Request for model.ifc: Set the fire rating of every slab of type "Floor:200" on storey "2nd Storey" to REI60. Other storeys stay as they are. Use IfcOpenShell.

First a look at what the model holds.

```python
import ifcopenshell
import ifcopenshell.util.element

model = ifcopenshell.open("model.ifc")
print(model.schema)
storey = next(s for s in model.by_type("IfcBuildingStorey") if s.Name == "2nd Storey")
slabs = [e for e in ifcopenshell.util.element.get_decomposition(storey) if e.is_a("IfcSlab")]
seen = {}
for e in slabs:
    element_type = ifcopenshell.util.element.get_type(e)
    key = (element_type.Name if element_type != e and element_type else None, ifcopenshell.util.element.get_pset(e, "Pset_SlabCommon", "FireRating"))
    seen[key] = seen.get(key, 0) + 1
for (name, value), count in sorted(seen.items(), key=str):
    print(count, "x", name, "|", value)
```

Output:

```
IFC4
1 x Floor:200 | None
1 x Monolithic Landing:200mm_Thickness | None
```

```python
import ifcopenshell
import ifcopenshell.api.pset
import ifcopenshell.util.element

model = ifcopenshell.open("model.ifc")

storey = next(s for s in model.by_type("IfcBuildingStorey") if s.Name == "2nd Storey")
slabs = [e for e in ifcopenshell.util.element.get_decomposition(storey) if e.is_a("IfcSlab")]

count = 0
for e in slabs:
    element_type = ifcopenshell.util.element.get_type(e)
    if element_type in (None, e) or element_type.Name != "Floor:200":
        continue
    # add_pset returns the element's existing set when there is one.
    pset = ifcopenshell.api.pset.add_pset(model, product=e, name="Pset_SlabCommon")
    ifcopenshell.api.pset.edit_pset(model, pset=pset, properties={"FireRating": "REI60"})
    count += 1

print(count, "slabs updated")

model.write("model_edited.ifc")
```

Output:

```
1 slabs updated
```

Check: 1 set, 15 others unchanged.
